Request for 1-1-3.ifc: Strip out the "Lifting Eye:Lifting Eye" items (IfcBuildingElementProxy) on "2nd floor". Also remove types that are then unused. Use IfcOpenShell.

First a look at what the model holds.

```python
import ifcopenshell
import ifcopenshell.util.element

model = ifcopenshell.open("1-1-3.ifc")
print(model.schema)
storey = next(s for s in model.by_type("IfcBuildingStorey") if s.Name == "2nd floor")
proxies = [e for e in ifcopenshell.util.element.get_decomposition(storey) if e.is_a("IfcBuildingElementProxy")]
seen = {}
for e in proxies:
    element_type = ifcopenshell.util.element.get_type(e)
    name = element_type.Name if element_type not in (None, e) else None
    seen[name] = seen.get(name, 0) + 1
for name, count in sorted(seen.items(), key=str):
    print(count, "x", name)
```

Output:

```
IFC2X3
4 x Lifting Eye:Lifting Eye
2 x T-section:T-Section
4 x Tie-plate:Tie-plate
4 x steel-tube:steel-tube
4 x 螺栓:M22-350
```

```python
import ifcopenshell
import ifcopenshell.api.root
import ifcopenshell.util.element

model = ifcopenshell.open("1-1-3.ifc")

storey = next(s for s in model.by_type("IfcBuildingStorey") if s.Name == "2nd floor")
proxies = [e for e in ifcopenshell.util.element.get_decomposition(storey) if e.is_a("IfcBuildingElementProxy")]
targets = [e for e in proxies if (t := ifcopenshell.util.element.get_type(e)) not in (None, e) and t.Name == "Lifting Eye:Lifting Eye"]
types = {ifcopenshell.util.element.get_type(e) for e in targets} - {None, *targets}

for e in targets:
    ifcopenshell.api.root.remove_product(model, product=e)
print(len(targets), "removed")

unused = [t for t in types if not ifcopenshell.util.element.get_types(t)]
for t in unused:
    ifcopenshell.api.root.remove_product(model, product=t)
print(len(unused), "unused types removed")

model.write("1-1-3_updated.ifc")
```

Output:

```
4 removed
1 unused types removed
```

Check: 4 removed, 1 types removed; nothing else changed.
